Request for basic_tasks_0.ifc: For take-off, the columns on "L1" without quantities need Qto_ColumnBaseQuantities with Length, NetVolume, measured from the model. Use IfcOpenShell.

First a look at what the model holds.

```python
import ifcopenshell
import ifcopenshell.util.element
import ifcopenshell.util.unit

model = ifcopenshell.open("basic_tasks_0.ifc")
print(model.schema)
for unit_type in ("LENGTHUNIT", "AREAUNIT", "VOLUMEUNIT"):
    print(unit_type, ifcopenshell.util.unit.calculate_unit_scale(model, unit_type))
storey = next(s for s in model.by_type("IfcBuildingStorey") if s.Name == "L1")
columns = [e for e in ifcopenshell.util.element.get_decomposition(storey) if e.is_a("IfcColumn")]
for e in sorted(columns, key=lambda e: e.id()):
    print(e.id(), e.is_a(), e.Name, list(ifcopenshell.util.element.get_psets(e, qtos_only=True)), sep=" | ")
```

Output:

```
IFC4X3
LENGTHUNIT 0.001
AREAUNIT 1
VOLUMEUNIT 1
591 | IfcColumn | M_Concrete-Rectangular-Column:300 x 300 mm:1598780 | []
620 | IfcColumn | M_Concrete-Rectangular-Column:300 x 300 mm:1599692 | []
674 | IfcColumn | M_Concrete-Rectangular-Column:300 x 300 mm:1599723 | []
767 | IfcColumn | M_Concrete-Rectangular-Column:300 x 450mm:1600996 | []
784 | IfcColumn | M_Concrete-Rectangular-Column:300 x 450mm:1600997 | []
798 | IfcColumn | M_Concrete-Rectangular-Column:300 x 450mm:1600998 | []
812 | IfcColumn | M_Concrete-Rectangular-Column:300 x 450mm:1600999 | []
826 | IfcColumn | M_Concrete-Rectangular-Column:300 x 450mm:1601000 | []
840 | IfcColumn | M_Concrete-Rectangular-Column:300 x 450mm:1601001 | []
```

```python
import ifcopenshell
import ifcopenshell.api.pset
import ifcopenshell.geom
import ifcopenshell.util.element
import ifcopenshell.util.shape
import ifcopenshell.util.unit

model = ifcopenshell.open("basic_tasks_0.ifc")
unit_scale = ifcopenshell.util.unit.calculate_unit_scale(model)
volume_scale = ifcopenshell.util.unit.calculate_unit_scale(model, "VOLUMEUNIT")
settings = ifcopenshell.geom.settings()

storey = next(s for s in model.by_type("IfcBuildingStorey") if s.Name == "L1")
columns = [e for e in ifcopenshell.util.element.get_decomposition(storey) if e.is_a("IfcColumn")]

for e in sorted(columns, key=lambda e: e.id()):
    if ifcopenshell.util.element.get_psets(e, qtos_only=True, should_inherit=False):
        continue
    # Geometry comes back in metres, in the element's own axes.
    shape = ifcopenshell.geom.create_shape(settings, e)
    values = {
        "Length": ifcopenshell.util.shape.get_z(shape.geometry) / unit_scale,
        "NetVolume": ifcopenshell.util.shape.get_volume(shape.geometry) / volume_scale,
    }
    qto = ifcopenshell.api.pset.add_qto(model, product=e, name="Qto_ColumnBaseQuantities")
    ifcopenshell.api.pset.edit_qto(model, qto=qto, properties=values)
    print(e.id(), {k: round(v, 3) for k, v in values.items()})

model.write("basic_tasks_0_updated.ifc")
```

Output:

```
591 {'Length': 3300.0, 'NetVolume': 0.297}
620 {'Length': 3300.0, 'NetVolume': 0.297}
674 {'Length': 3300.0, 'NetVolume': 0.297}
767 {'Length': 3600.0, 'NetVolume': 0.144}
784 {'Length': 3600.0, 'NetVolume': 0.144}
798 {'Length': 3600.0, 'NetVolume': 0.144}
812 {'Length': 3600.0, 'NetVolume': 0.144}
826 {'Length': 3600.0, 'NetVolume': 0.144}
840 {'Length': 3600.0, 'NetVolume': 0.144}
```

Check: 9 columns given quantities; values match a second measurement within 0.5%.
